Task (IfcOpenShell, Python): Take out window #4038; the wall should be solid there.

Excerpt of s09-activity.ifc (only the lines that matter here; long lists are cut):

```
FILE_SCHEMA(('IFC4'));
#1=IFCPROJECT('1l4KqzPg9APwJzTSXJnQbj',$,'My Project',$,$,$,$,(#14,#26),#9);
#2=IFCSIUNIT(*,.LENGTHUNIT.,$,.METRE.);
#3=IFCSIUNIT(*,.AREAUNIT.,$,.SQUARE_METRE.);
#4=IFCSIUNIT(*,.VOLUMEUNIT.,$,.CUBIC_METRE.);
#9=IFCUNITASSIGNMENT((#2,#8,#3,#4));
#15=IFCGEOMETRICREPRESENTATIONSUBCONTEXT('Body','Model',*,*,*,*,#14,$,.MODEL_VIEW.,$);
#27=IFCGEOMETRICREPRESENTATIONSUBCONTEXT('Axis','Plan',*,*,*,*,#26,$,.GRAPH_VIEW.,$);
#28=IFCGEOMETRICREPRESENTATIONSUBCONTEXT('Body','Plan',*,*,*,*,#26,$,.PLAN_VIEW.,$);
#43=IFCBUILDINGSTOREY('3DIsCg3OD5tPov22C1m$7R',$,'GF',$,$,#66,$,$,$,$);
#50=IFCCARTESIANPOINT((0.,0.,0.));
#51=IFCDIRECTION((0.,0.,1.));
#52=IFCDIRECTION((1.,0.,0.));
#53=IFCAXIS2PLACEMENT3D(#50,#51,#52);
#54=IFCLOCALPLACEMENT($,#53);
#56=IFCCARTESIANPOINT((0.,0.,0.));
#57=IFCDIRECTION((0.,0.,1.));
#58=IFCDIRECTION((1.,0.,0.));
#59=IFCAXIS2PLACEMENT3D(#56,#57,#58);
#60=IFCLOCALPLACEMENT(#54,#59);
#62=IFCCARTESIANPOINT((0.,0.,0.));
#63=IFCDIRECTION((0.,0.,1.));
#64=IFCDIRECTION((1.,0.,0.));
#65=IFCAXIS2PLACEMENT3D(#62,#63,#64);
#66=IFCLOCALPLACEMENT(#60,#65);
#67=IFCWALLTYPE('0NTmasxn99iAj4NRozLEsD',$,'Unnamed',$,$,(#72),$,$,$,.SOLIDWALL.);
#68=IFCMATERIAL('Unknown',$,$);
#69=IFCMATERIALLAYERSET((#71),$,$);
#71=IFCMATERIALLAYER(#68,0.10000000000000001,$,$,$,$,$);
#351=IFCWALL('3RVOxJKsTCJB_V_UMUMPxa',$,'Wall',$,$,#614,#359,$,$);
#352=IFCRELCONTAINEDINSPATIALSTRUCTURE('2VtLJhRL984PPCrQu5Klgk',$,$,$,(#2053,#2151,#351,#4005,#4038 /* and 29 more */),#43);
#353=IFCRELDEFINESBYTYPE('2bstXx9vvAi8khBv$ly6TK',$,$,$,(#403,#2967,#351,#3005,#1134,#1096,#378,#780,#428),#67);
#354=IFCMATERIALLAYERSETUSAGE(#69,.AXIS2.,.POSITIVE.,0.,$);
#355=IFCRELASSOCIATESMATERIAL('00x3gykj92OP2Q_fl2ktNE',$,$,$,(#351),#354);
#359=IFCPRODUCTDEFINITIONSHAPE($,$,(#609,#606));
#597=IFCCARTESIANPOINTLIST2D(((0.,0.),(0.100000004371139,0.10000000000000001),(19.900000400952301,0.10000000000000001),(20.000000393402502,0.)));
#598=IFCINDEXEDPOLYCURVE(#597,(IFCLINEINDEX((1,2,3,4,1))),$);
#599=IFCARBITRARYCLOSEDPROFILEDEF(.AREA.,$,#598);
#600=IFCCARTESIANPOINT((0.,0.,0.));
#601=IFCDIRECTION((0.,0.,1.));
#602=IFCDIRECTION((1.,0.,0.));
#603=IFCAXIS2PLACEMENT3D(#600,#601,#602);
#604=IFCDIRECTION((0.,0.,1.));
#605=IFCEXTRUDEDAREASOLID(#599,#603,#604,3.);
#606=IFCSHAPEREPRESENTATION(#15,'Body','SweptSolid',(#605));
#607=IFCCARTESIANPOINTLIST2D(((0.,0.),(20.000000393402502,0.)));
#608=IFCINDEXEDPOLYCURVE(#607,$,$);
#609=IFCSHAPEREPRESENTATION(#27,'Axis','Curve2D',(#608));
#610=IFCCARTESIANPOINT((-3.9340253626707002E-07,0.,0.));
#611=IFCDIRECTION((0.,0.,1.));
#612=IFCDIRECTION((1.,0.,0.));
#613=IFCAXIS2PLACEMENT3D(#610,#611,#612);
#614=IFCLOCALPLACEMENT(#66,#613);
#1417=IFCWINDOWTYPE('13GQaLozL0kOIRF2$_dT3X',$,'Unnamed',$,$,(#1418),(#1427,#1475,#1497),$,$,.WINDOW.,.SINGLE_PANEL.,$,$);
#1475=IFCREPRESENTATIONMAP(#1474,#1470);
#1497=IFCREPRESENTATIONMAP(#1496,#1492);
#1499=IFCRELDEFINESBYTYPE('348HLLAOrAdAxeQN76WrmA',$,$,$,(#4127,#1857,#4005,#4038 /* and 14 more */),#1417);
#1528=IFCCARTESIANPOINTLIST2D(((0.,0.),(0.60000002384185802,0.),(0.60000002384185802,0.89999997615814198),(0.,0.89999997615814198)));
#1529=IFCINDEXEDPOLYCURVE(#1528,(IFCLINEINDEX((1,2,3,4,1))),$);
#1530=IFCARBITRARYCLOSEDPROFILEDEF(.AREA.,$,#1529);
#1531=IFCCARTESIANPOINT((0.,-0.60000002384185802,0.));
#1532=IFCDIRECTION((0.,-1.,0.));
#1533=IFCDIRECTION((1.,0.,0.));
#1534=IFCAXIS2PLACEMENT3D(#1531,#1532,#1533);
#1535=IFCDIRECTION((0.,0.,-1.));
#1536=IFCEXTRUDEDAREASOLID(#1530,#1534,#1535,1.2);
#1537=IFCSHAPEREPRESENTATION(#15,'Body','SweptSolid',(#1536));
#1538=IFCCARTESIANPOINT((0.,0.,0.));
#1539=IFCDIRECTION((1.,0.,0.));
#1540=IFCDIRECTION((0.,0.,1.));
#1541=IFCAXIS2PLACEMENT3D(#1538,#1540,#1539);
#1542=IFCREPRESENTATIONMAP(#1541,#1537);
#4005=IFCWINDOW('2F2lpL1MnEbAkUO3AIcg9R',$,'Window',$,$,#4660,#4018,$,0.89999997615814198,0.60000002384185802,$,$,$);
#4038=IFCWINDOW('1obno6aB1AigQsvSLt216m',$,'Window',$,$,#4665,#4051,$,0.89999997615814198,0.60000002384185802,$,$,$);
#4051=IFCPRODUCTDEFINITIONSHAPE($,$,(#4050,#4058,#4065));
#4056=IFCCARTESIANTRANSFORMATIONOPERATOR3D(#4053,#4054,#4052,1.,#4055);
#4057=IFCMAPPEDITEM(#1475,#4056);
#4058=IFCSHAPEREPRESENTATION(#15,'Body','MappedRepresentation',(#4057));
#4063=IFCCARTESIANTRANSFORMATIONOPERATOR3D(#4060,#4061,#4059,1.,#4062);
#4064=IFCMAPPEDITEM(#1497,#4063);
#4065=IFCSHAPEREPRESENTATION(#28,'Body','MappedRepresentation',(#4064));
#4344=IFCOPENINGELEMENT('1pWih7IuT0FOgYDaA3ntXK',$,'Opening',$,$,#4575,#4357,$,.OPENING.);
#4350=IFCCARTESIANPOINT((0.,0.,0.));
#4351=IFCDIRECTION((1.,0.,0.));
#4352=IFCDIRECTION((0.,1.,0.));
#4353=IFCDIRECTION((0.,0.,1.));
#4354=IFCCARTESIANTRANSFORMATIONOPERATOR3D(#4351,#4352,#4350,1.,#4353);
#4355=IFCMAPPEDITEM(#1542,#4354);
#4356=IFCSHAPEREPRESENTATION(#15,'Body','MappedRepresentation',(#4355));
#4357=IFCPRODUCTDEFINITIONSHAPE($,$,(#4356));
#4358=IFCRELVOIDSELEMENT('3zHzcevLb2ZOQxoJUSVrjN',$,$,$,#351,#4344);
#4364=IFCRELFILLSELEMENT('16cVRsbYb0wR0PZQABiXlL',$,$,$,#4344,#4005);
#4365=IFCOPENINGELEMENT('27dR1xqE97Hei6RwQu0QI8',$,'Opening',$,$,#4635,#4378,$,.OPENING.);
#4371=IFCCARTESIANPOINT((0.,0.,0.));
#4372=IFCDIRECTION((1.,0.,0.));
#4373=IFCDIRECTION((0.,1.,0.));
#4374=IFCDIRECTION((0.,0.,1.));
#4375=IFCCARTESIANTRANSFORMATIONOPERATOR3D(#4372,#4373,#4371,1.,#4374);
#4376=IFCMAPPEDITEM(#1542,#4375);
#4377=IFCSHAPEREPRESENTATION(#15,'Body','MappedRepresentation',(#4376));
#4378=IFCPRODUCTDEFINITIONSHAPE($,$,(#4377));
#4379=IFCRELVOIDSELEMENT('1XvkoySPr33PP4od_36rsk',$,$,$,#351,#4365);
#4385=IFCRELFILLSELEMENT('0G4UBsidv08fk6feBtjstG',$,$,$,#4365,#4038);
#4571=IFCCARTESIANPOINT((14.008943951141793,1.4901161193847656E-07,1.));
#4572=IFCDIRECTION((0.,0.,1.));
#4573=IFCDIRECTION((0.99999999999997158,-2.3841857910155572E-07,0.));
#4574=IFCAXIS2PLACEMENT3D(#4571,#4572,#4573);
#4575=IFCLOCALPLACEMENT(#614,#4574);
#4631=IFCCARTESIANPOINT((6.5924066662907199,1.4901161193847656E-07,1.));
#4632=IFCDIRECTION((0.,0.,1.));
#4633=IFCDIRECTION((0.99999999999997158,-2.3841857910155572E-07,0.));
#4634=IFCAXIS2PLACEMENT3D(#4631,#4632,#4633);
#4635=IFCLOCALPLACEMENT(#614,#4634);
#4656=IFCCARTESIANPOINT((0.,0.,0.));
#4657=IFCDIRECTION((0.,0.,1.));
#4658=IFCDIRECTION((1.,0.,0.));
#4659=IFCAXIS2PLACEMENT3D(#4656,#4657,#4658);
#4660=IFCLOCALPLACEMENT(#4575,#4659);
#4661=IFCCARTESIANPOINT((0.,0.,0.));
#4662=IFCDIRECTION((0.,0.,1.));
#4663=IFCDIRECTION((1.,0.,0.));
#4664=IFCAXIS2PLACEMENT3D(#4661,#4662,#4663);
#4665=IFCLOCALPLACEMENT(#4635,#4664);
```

```python
import ifcopenshell
import ifcopenshell.api.feature
import ifcopenshell.api.root
import ifcopenshell.geom
import ifcopenshell.util.shape

model = ifcopenshell.open("s09-activity.ifc")
settings = ifcopenshell.geom.settings()


def volume(element):
    """Net volume in cubic metres, openings subtracted."""
    shape = ifcopenshell.geom.create_shape(settings, element)
    return ifcopenshell.util.shape.get_volume(shape.geometry)


window = model.by_guid("1obno6aB1AigQsvSLt216m")
opening = window.FillsVoids[0].RelatingOpeningElement
wall = opening.VoidsElements[0].RelatingBuildingElement
before = volume(wall)

ifcopenshell.api.root.remove_product(model, product=window)
ifcopenshell.api.feature.remove_feature(model, feature=opening)

after = volume(wall)

print(f"wall volume {before:.3f} -> {after:.3f} m3")

model.write("s09-activity_v2.ifc")
```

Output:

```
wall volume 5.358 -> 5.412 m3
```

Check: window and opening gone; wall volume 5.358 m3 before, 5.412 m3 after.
